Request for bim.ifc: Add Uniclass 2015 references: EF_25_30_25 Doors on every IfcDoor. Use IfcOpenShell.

First a look at what the model holds.

```python
import ifcopenshell

model = ifcopenshell.open("bim.ifc")
print(model.schema)
print("classifications:", [c.Name for c in model.by_type("IfcClassification")])
for ifc_class in ("IfcDoor", "IfcRoof", "IfcStair", "IfcWall", "IfcWindow"):
    print(ifc_class, len(model.by_type(ifc_class)))
```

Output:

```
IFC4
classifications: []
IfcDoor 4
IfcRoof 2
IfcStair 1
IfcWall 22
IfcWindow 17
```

```python
import ifcopenshell
import ifcopenshell.api.classification

model = ifcopenshell.open("bim.ifc")

system = ifcopenshell.api.classification.add_classification(model, classification="Uniclass 2015")

codes = {
    "IfcDoor": ("EF_25_30_25", "Doors"),
}
for ifc_class, (code, name) in codes.items():
    products = model.by_type(ifc_class)
    ifcopenshell.api.classification.add_reference(
        model, products=products, classification=system, identification=code, name=name
    )
    print(code, len(products))

model.write("bim_rev.ifc")
```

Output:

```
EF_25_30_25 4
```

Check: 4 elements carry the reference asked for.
